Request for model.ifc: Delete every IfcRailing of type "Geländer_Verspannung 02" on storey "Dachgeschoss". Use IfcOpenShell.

First a look at what the model holds.

```python
import ifcopenshell
import ifcopenshell.util.element

model = ifcopenshell.open("model.ifc")
print(model.schema)
storey = next(s for s in model.by_type("IfcBuildingStorey") if s.Name == "Dachgeschoss")
railings = [e for e in ifcopenshell.util.element.get_decomposition(storey) if e.is_a("IfcRailing")]
seen = {}
for e in railings:
    element_type = ifcopenshell.util.element.get_type(e)
    name = element_type.Name if element_type not in (None, e) else None
    seen[name] = seen.get(name, 0) + 1
for name, count in sorted(seen.items(), key=str):
    print(count, "x", name)
```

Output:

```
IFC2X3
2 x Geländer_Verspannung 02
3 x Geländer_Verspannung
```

```python
import ifcopenshell
import ifcopenshell.api.root
import ifcopenshell.util.element

model = ifcopenshell.open("model.ifc")

storey = next(s for s in model.by_type("IfcBuildingStorey") if s.Name == "Dachgeschoss")
railings = [e for e in ifcopenshell.util.element.get_decomposition(storey) if e.is_a("IfcRailing")]
targets = [e for e in railings if (t := ifcopenshell.util.element.get_type(e)) not in (None, e) and t.Name == "Geländer_Verspannung 02"]

for e in targets:
    ifcopenshell.api.root.remove_product(model, product=e)
print(len(targets), "removed")

model.write("model_rev.ifc")
```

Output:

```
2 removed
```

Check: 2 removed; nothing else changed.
